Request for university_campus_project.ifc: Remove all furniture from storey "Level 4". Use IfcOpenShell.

First a look at what the model holds.

```python
import ifcopenshell
import ifcopenshell.util.element

model = ifcopenshell.open("university_campus_project.ifc")
print(model.schema)
storey = next(s for s in model.by_type("IfcBuildingStorey") if s.Name == "Level 4")
furniture = [e for e in ifcopenshell.util.element.get_decomposition(storey) if e.is_a("IfcFurnishingElement")]
seen = {}
for e in furniture:
    element_type = ifcopenshell.util.element.get_type(e)
    name = element_type.Name if element_type not in (None, e) else None
    seen[name] = seen.get(name, 0) + 1
for name, count in sorted(seen.items(), key=str):
    print(count, "x", name)
```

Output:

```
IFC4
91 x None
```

```python
import ifcopenshell
import ifcopenshell.api.root
import ifcopenshell.util.element

model = ifcopenshell.open("university_campus_project.ifc")

storey = next(s for s in model.by_type("IfcBuildingStorey") if s.Name == "Level 4")
furniture = [e for e in ifcopenshell.util.element.get_decomposition(storey) if e.is_a("IfcFurnishingElement")]

for e in furniture:
    ifcopenshell.api.root.remove_product(model, product=e)
print(len(furniture), "removed")

model.write("university_campus_project-out.ifc")
```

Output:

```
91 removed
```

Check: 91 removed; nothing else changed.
